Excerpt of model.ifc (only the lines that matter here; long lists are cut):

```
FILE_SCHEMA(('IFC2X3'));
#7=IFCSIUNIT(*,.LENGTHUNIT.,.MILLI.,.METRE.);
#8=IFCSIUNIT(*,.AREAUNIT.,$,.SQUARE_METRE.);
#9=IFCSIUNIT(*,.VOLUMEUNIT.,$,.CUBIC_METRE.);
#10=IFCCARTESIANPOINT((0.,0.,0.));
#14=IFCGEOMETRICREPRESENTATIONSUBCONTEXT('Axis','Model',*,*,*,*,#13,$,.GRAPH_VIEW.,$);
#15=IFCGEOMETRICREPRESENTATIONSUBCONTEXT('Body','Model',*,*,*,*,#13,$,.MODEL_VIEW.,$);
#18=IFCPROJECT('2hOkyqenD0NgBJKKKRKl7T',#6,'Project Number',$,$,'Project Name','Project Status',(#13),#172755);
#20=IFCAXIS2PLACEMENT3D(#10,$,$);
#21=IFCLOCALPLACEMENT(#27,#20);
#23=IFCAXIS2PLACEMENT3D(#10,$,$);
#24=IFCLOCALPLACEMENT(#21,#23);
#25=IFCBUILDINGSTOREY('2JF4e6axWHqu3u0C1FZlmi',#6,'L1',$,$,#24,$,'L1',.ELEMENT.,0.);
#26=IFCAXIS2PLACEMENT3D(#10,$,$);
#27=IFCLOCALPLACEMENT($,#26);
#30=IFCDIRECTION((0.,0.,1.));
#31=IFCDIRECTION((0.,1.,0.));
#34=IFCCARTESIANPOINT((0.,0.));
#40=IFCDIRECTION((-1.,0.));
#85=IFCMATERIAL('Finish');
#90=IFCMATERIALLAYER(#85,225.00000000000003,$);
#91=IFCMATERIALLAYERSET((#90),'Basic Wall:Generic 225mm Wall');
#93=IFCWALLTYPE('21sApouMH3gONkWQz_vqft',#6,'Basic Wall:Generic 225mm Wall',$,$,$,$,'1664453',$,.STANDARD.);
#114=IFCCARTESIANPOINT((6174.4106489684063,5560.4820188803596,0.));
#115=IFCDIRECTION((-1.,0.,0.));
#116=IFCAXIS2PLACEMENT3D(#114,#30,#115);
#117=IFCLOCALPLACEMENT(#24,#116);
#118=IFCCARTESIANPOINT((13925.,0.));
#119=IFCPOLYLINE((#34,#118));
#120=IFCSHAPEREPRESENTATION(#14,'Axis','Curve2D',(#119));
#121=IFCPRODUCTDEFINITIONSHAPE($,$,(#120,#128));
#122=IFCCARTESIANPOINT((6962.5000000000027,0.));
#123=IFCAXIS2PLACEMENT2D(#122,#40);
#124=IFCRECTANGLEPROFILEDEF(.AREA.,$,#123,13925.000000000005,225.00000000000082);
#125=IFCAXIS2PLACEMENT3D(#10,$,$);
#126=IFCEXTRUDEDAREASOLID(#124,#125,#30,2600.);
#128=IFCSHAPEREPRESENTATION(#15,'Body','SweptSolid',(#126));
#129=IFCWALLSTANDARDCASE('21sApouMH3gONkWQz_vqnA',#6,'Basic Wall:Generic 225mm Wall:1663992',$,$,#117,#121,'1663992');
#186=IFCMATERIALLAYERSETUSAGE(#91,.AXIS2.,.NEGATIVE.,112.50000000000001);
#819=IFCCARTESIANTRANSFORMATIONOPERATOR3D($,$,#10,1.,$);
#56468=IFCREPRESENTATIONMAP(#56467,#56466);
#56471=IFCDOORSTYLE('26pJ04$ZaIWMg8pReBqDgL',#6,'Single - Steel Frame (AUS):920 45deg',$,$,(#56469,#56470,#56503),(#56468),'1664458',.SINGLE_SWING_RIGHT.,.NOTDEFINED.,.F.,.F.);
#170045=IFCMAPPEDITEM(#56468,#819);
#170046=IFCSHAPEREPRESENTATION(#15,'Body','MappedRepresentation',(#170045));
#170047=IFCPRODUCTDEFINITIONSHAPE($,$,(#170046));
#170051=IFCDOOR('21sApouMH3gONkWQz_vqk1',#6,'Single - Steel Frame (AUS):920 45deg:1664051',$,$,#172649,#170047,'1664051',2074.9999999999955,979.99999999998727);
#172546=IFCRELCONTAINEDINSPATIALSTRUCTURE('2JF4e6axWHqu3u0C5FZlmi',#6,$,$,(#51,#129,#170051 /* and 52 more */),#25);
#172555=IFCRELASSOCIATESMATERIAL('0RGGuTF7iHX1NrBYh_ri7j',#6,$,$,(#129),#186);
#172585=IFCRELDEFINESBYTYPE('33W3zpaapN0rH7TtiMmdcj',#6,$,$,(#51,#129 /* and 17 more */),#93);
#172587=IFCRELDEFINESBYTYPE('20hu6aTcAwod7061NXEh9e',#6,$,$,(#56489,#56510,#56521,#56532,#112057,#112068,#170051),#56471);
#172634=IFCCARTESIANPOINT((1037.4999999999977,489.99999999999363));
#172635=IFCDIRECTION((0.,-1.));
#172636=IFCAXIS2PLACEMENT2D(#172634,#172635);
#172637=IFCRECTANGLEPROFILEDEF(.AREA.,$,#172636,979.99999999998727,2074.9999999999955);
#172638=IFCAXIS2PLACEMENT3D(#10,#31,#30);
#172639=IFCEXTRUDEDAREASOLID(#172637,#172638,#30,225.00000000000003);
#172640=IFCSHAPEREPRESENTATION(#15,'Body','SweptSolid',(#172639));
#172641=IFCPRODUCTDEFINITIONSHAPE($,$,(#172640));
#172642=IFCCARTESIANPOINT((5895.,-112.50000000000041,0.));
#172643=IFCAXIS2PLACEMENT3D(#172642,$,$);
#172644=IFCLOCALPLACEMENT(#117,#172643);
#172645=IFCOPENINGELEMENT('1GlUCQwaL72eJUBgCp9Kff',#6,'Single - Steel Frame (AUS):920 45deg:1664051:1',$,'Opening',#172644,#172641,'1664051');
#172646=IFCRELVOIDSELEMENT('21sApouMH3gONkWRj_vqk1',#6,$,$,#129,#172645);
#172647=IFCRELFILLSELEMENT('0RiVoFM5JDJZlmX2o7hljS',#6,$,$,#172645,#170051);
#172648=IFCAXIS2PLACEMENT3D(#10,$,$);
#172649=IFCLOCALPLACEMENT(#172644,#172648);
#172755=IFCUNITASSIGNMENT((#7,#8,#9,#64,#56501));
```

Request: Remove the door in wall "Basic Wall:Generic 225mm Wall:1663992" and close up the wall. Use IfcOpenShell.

```python
import ifcopenshell
import ifcopenshell.api.feature
import ifcopenshell.api.root
import ifcopenshell.geom
import ifcopenshell.util.shape

model = ifcopenshell.open("model.ifc")
settings = ifcopenshell.geom.settings()


def volume(element):
    """Net volume in cubic metres, openings subtracted."""
    shape = ifcopenshell.geom.create_shape(settings, element)
    return ifcopenshell.util.shape.get_volume(shape.geometry)


door = model.by_guid("21sApouMH3gONkWQz_vqk1")
opening = door.FillsVoids[0].RelatingOpeningElement
wall = opening.VoidsElements[0].RelatingBuildingElement
before = volume(wall)

ifcopenshell.api.root.remove_product(model, product=door)
ifcopenshell.api.feature.remove_feature(model, feature=opening)

after = volume(wall)

print(f"wall volume {before:.3f} -> {after:.3f} m3")

model.write("model_rev.ifc")
```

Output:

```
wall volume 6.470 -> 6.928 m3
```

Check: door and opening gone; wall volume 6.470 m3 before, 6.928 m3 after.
